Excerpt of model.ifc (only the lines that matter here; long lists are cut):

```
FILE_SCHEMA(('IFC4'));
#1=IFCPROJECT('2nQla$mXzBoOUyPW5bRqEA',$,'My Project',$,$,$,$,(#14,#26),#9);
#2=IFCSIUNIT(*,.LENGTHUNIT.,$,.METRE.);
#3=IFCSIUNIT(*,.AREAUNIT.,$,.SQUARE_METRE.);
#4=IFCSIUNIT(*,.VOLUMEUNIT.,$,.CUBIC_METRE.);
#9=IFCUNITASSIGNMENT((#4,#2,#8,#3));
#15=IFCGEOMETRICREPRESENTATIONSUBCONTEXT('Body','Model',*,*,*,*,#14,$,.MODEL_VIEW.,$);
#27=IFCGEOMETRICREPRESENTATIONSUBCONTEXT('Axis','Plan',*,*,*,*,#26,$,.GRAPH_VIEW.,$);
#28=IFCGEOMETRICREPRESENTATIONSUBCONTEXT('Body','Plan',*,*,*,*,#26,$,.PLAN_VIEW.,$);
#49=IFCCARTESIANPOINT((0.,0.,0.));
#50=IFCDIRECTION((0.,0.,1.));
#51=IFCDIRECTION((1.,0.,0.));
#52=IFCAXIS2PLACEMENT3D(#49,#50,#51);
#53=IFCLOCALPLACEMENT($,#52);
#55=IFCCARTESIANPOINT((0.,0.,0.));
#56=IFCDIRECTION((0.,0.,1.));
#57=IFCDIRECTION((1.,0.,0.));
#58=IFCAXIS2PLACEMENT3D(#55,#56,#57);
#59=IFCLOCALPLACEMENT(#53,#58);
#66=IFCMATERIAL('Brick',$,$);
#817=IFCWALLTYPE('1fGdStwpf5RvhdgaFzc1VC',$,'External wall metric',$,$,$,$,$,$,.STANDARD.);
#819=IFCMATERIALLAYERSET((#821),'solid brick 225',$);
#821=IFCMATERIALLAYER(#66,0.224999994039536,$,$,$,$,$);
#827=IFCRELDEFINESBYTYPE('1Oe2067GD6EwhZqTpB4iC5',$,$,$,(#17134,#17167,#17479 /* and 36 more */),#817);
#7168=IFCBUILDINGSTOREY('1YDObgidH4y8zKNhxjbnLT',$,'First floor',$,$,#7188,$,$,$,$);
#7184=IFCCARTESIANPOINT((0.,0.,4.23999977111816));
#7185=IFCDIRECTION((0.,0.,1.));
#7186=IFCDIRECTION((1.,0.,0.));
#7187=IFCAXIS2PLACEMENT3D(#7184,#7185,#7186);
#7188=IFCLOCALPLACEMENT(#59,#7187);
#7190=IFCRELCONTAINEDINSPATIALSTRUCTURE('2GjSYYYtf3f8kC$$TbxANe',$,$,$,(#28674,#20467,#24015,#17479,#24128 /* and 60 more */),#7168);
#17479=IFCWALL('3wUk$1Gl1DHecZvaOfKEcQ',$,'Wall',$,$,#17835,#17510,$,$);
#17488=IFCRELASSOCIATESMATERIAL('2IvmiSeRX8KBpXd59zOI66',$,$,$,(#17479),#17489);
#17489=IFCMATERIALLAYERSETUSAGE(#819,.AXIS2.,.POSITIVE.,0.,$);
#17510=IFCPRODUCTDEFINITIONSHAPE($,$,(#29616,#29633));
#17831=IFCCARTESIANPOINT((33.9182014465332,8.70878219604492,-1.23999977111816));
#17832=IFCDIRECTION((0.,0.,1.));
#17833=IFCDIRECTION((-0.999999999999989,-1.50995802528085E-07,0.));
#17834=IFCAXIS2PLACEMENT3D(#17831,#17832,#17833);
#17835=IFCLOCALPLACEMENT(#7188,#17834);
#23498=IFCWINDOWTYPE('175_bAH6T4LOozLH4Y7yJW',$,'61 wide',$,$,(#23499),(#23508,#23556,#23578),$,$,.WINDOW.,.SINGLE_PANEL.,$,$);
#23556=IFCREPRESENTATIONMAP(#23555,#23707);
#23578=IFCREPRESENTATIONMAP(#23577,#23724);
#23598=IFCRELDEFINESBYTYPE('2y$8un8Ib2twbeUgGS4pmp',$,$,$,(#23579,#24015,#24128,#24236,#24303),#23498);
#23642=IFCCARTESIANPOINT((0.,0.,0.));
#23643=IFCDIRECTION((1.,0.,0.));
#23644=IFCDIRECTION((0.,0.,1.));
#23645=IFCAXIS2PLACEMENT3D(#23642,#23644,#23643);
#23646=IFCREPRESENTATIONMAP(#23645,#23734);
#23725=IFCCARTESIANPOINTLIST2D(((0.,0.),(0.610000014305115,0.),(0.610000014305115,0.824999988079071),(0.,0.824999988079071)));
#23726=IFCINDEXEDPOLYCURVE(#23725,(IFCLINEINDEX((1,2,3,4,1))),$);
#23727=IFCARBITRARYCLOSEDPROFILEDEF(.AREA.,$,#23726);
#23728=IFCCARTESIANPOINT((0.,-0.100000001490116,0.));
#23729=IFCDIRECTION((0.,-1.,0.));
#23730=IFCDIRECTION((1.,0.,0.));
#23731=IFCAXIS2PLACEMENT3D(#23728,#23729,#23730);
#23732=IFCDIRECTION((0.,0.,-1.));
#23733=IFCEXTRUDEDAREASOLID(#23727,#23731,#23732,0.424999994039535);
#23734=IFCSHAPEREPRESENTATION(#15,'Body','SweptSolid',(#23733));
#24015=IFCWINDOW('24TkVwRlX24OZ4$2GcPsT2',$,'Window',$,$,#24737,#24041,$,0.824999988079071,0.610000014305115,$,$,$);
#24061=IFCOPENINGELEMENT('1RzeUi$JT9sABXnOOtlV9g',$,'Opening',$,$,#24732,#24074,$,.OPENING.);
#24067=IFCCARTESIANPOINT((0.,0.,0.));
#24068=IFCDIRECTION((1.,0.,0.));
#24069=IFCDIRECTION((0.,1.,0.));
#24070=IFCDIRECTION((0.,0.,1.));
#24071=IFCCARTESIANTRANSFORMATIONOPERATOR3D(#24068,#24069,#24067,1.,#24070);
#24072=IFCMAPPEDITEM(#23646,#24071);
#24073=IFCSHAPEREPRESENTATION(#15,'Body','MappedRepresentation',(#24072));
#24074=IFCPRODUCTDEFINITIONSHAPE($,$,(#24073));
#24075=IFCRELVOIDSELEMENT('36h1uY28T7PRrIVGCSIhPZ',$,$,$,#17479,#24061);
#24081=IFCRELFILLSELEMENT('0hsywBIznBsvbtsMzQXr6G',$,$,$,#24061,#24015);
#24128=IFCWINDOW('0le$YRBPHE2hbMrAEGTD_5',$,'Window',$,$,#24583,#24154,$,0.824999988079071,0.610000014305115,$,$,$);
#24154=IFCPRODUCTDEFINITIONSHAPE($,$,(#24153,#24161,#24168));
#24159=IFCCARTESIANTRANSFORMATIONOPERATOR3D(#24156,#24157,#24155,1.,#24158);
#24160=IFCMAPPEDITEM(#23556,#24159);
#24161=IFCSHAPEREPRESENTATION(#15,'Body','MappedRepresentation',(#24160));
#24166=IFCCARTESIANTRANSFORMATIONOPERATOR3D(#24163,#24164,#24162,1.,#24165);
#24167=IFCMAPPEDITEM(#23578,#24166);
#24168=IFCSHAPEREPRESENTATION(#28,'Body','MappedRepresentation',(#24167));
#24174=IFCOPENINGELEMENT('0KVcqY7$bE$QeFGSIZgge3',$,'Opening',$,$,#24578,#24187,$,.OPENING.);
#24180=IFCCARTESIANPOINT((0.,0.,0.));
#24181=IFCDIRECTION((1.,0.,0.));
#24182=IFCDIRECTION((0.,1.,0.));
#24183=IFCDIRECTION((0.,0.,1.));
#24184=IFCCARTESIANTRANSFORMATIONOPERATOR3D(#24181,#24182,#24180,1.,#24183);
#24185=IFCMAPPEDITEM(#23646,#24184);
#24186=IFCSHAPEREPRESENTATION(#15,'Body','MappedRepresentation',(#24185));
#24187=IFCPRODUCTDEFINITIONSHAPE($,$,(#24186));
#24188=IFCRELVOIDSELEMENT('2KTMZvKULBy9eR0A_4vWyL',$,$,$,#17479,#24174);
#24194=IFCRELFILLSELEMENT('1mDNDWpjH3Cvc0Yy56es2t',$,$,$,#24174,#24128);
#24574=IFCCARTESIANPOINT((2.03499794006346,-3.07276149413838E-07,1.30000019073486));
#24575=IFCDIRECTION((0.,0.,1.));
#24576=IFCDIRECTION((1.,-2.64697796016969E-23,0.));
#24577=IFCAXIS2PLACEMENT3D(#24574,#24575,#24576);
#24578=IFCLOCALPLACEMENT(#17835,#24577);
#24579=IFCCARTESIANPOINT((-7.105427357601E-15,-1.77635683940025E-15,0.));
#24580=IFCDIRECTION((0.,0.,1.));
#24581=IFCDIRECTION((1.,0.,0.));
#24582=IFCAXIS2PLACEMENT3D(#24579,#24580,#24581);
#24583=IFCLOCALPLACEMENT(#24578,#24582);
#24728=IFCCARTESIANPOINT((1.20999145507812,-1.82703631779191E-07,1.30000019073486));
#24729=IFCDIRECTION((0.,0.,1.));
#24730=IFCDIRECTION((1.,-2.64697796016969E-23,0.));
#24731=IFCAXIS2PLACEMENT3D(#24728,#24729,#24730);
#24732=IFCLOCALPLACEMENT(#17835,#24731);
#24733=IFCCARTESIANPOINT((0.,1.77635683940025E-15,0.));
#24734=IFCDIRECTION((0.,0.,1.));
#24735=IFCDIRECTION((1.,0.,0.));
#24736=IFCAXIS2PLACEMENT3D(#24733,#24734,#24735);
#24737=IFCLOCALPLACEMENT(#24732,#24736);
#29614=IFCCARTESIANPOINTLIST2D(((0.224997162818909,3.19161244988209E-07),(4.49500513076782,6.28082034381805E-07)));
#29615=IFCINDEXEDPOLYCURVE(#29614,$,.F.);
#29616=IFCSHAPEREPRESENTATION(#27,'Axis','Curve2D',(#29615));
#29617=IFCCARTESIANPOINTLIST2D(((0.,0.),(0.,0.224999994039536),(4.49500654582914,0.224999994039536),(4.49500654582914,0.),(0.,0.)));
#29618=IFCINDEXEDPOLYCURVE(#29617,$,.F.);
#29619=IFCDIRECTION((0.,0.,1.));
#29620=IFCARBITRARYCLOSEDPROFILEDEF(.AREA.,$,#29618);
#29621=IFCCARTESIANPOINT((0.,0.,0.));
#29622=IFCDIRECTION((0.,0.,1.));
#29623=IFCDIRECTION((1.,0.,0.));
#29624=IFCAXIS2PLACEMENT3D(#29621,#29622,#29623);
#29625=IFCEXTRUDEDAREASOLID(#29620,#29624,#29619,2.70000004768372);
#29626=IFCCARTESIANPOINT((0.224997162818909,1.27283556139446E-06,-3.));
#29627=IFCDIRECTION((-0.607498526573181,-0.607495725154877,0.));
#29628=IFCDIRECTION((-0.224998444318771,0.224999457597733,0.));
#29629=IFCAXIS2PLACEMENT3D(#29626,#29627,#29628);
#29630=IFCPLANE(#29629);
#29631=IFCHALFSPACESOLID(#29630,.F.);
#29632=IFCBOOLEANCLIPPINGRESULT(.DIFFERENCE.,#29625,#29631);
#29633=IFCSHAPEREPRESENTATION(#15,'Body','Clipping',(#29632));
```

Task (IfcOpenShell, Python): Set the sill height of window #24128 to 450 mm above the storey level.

```python
import numpy as np
import ifcopenshell
import ifcopenshell.api.geometry
import ifcopenshell.geom
import ifcopenshell.util.element
import ifcopenshell.util.placement
import ifcopenshell.util.shape
import ifcopenshell.util.unit

model = ifcopenshell.open("model.ifc")
unit_scale = ifcopenshell.util.unit.calculate_unit_scale(model)

window = model.by_id(24128)
opening = window.FillsVoids[0].RelatingOpeningElement
storey = ifcopenshell.util.element.get_container(window, ifc_class="IfcBuildingStorey")
level = ifcopenshell.util.placement.get_local_placement(storey.ObjectPlacement)[2, 3]

# The opening's origin need not be at the sill, so measure its lowest point.
shape = ifcopenshell.geom.create_shape(ifcopenshell.geom.settings(), opening)
bottom = ifcopenshell.util.shape.get_shape_bottom_elevation(shape, shape.geometry) / unit_scale
dz = level + 0.45 / unit_scale - bottom

shift = np.array([0.0, 0.0, dz])
# The window is placed relative to its opening, so it follows when the opening moves.
matrix = ifcopenshell.util.placement.get_local_placement(opening.ObjectPlacement)
matrix[:3, 3] += shift
ifcopenshell.api.geometry.edit_object_placement(
    model, product=opening, matrix=matrix, is_si=False, should_transform_children=True
)

print(f"moved by {dz * unit_scale:+.3f} m")

model.write("model_v2.ifc")
```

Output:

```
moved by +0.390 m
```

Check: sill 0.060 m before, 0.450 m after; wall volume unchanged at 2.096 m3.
